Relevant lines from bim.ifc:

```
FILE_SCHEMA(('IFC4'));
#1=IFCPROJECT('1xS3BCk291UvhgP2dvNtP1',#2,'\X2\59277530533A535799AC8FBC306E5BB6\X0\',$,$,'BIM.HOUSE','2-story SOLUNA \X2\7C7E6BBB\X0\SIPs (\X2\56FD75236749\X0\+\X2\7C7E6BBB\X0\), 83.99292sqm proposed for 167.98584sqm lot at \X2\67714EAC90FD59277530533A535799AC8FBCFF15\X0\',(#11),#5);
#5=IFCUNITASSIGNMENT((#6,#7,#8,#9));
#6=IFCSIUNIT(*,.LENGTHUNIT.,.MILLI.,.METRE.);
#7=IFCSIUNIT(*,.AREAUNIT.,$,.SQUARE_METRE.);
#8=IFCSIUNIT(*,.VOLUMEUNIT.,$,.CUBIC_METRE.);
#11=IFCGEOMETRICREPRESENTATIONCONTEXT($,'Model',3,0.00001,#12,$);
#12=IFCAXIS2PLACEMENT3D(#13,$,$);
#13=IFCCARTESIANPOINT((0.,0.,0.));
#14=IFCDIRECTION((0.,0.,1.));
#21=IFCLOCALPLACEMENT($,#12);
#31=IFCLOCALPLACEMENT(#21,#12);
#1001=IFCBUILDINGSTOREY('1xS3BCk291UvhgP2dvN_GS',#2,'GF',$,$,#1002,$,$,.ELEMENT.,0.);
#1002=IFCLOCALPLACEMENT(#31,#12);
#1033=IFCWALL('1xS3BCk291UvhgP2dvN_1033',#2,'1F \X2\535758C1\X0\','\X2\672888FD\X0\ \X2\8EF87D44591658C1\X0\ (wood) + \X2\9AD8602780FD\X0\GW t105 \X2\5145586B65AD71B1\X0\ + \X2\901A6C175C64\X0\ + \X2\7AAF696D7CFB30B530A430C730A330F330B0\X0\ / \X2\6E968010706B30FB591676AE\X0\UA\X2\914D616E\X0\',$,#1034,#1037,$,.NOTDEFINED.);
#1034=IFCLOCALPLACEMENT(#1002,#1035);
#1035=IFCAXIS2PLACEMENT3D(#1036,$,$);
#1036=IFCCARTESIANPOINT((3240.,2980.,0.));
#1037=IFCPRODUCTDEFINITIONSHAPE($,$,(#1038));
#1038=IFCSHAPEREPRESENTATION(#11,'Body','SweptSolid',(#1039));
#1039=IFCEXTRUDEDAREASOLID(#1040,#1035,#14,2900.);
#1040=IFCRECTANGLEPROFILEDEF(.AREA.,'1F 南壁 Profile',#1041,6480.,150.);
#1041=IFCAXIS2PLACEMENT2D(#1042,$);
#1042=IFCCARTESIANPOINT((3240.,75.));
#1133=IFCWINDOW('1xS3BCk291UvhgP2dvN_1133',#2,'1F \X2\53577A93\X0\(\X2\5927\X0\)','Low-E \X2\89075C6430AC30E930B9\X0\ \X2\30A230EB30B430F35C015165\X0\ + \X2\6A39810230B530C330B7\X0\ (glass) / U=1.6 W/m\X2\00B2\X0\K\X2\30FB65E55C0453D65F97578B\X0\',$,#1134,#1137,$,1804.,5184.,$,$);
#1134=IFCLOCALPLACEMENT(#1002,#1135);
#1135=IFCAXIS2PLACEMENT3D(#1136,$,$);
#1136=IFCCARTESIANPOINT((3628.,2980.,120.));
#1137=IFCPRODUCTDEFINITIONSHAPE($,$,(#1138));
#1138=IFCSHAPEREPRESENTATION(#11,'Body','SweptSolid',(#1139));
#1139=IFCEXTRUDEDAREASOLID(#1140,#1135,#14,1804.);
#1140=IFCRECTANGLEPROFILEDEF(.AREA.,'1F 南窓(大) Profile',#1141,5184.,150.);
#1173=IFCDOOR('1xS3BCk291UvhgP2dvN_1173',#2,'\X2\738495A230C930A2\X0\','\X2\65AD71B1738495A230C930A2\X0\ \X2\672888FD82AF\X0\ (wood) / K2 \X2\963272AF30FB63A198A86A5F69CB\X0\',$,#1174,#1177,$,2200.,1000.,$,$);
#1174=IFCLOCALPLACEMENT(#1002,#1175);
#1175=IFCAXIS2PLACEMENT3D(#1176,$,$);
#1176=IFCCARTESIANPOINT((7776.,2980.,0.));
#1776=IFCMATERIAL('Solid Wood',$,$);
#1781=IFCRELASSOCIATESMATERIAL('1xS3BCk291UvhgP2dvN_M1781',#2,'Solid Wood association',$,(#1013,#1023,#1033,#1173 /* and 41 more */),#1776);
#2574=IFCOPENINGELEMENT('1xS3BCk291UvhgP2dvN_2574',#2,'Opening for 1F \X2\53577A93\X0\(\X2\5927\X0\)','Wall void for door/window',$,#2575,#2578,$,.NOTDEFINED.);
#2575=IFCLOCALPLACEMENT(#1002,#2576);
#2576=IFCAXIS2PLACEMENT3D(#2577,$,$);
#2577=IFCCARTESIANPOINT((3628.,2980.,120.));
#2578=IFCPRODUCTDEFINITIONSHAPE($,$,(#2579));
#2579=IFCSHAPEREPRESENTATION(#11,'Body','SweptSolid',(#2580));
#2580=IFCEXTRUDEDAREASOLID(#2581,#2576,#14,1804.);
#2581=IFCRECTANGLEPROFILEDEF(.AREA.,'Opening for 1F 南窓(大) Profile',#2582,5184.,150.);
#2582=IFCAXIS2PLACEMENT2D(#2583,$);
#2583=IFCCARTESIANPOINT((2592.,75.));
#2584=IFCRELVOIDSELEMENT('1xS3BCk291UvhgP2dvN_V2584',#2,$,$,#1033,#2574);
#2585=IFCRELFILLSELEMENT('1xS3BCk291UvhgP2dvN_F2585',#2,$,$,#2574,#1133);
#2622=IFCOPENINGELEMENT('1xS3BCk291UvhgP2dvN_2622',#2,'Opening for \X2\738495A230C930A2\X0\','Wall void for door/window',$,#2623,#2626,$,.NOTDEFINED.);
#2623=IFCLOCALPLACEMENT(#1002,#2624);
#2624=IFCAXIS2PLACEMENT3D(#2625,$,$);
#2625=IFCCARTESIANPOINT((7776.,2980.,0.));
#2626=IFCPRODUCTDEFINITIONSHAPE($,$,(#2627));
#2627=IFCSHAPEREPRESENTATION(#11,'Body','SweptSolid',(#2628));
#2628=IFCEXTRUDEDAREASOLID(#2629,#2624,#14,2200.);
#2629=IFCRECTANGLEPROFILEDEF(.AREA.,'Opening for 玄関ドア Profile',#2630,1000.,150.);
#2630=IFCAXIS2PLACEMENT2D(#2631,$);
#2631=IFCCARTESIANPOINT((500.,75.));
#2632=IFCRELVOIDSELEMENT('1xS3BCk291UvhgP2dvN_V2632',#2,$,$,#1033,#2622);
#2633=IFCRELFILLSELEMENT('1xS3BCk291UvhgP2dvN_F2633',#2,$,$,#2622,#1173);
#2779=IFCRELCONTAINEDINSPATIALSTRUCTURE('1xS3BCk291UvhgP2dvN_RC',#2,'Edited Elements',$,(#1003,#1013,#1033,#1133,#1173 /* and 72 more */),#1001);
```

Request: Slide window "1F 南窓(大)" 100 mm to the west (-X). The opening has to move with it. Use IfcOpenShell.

```python
import ifcopenshell
import ifcopenshell.api.geometry
import ifcopenshell.util.placement

model = ifcopenshell.open("bim.ifc")

window = model.by_guid("1xS3BCk291UvhgP2dvN_1133")
opening = window.FillsVoids[0].RelatingOpeningElement
wall = opening.VoidsElements[0].RelatingBuildingElement

wall_matrix = ifcopenshell.util.placement.get_local_placement(wall.ObjectPlacement)
shift = wall_matrix[:3, 0] * -100.0
before = ifcopenshell.util.placement.get_local_placement(window.ObjectPlacement)[:3, 3].copy()

# The window is not placed relative to its opening, so move both.
for product in (opening, window):
    matrix = ifcopenshell.util.placement.get_local_placement(product.ObjectPlacement)
    matrix[:3, 3] += shift
    ifcopenshell.api.geometry.edit_object_placement(model, product=product, matrix=matrix, is_si=False)

after = ifcopenshell.util.placement.get_local_placement(window.ObjectPlacement)[:3, 3]
print("window moved by", (after - before).round(3) + 0.0)

model.write("bim_rev.ifc")
```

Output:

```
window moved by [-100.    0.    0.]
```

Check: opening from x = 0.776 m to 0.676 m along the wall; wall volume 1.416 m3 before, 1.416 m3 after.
